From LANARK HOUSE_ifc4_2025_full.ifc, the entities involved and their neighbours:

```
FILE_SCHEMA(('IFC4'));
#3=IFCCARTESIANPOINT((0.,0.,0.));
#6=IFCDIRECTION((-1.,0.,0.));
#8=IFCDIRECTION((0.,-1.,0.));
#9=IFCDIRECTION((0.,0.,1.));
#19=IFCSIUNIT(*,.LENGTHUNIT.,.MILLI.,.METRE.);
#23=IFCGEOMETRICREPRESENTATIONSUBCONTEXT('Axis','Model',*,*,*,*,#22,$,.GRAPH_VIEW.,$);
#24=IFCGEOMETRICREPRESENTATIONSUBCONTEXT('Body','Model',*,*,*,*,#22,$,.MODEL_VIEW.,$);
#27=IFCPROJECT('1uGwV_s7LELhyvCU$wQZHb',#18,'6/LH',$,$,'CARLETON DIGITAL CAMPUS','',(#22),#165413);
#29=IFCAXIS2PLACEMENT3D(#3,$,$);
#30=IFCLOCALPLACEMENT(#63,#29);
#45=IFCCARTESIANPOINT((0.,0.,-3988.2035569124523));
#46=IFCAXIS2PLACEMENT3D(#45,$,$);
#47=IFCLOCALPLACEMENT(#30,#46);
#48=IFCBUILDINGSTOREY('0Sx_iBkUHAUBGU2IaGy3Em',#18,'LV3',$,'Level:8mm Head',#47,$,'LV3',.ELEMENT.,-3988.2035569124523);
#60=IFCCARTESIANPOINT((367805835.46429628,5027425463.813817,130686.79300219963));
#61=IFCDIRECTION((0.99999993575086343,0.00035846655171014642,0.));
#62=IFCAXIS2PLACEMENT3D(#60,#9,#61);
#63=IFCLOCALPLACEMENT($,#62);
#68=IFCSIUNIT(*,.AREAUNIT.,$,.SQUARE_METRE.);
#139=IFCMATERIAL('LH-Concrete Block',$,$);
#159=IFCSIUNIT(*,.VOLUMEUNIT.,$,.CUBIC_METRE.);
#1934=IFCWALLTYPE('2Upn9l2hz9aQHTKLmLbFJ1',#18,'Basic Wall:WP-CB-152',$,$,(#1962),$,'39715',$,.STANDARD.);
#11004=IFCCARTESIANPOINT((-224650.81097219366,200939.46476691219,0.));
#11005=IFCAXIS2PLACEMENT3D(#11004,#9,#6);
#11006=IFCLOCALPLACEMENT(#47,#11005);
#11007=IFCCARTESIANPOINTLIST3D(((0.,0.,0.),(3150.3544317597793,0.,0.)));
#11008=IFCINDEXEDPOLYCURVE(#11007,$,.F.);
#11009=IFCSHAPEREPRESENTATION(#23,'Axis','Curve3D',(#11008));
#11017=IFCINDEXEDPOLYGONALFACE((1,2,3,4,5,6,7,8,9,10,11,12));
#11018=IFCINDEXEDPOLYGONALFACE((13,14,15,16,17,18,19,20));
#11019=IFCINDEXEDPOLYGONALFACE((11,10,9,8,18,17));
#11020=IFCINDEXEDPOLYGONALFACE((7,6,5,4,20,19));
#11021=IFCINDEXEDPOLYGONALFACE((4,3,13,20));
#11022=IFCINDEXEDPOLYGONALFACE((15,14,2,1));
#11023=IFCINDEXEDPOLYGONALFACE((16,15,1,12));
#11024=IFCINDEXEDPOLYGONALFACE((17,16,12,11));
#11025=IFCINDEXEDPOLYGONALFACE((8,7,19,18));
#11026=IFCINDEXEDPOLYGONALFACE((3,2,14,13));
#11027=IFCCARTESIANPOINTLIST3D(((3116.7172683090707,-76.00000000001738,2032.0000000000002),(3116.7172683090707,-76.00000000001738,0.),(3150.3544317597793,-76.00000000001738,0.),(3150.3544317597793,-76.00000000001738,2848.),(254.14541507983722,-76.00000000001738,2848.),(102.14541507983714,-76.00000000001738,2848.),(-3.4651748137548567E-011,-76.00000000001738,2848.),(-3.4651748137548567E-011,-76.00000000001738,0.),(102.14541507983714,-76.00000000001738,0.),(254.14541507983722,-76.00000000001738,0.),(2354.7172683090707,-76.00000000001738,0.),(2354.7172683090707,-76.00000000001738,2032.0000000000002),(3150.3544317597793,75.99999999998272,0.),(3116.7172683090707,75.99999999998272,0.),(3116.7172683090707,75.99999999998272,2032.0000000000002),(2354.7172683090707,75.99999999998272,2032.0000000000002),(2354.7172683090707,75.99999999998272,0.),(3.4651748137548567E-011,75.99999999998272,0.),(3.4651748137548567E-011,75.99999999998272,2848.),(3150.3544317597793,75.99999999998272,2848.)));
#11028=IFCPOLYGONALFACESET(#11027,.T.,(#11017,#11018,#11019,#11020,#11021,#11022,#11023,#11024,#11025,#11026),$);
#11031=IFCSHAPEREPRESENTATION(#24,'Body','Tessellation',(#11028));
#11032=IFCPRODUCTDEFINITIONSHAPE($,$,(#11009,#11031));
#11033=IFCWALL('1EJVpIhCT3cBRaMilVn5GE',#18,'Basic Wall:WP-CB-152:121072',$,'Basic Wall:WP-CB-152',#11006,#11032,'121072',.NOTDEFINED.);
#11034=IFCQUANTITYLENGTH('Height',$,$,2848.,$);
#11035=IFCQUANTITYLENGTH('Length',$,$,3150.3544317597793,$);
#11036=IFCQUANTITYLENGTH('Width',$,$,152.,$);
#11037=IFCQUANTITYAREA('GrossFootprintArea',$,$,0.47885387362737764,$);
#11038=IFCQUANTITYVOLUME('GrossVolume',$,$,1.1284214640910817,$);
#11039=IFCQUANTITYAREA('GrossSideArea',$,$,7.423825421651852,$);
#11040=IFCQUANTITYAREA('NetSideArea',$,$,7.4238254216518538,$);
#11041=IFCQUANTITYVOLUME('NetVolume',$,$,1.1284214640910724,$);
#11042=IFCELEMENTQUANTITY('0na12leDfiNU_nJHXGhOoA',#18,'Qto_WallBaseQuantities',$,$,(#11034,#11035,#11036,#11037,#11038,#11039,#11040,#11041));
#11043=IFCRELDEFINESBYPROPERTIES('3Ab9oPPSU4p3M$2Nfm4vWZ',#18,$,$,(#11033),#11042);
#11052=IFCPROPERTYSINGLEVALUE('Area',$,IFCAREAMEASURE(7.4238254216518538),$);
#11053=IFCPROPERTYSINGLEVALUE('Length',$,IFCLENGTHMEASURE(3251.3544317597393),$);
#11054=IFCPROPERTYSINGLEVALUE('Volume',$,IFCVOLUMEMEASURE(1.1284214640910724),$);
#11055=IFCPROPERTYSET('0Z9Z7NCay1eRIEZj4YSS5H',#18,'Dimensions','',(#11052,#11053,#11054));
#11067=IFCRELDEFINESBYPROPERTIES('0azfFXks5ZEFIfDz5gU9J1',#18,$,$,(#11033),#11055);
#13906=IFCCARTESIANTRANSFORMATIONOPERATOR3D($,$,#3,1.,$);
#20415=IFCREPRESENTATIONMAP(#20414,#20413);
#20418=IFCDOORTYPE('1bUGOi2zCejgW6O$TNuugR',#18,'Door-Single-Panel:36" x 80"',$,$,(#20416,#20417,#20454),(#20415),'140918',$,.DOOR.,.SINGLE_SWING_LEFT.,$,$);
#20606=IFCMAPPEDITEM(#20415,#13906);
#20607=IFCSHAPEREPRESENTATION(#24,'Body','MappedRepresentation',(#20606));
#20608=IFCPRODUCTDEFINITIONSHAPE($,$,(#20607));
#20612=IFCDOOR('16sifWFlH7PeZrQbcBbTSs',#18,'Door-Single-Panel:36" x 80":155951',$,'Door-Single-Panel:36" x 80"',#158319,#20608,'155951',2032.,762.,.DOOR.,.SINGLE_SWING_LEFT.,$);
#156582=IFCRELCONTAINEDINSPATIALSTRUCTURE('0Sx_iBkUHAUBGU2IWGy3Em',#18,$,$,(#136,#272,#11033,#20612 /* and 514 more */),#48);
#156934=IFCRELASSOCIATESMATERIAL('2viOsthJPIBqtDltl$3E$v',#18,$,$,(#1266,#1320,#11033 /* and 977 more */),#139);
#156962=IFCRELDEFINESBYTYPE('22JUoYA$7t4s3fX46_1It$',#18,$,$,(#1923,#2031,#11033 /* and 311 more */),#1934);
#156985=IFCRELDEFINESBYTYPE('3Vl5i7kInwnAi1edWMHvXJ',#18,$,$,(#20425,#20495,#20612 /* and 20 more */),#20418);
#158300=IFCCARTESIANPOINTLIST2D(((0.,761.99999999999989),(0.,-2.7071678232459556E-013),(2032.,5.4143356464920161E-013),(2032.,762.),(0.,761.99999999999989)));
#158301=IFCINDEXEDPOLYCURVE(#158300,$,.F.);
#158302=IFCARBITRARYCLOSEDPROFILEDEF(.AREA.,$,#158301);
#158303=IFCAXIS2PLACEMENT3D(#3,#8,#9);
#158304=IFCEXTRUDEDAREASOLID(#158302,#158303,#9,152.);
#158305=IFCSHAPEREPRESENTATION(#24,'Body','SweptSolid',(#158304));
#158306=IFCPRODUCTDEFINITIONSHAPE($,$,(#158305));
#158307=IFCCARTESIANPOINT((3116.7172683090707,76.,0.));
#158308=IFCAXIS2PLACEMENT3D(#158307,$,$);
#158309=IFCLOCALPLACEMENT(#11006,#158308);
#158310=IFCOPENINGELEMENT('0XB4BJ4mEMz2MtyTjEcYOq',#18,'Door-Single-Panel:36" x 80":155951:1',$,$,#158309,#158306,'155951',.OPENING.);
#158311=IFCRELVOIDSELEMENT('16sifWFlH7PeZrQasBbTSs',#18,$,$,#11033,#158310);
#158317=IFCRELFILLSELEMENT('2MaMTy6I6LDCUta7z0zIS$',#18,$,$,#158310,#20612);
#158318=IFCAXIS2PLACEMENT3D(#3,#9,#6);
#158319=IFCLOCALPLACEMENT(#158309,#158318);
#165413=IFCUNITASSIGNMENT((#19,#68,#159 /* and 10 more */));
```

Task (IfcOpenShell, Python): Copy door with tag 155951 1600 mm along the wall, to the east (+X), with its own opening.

```python
import ifcopenshell
import ifcopenshell.api.feature
import ifcopenshell.api.geometry
import ifcopenshell.api.pset
import ifcopenshell.api.root
import ifcopenshell.geom
import ifcopenshell.util.element
import ifcopenshell.util.placement
import ifcopenshell.util.shape
import ifcopenshell.util.unit

model = ifcopenshell.open("LANARK HOUSE_ifc4_2025_full.ifc")
unit_scale = ifcopenshell.util.unit.calculate_unit_scale(model)
area_scale = ifcopenshell.util.unit.calculate_unit_scale(model, "AREAUNIT")
volume_scale = ifcopenshell.util.unit.calculate_unit_scale(model, "VOLUMEUNIT")
settings = ifcopenshell.geom.settings()


def volume(element):
    """Net volume in cubic metres, openings subtracted."""
    shape = ifcopenshell.geom.create_shape(settings, element)
    return ifcopenshell.util.shape.get_volume(shape.geometry)


def reuse_history(source, copy):
    """copy_class also copies each property set's owner history, people and application; keep the originals."""
    for rel in copy.IsDefinedBy:
        if rel.is_a("IfcRelDefinesByProperties") and (history := rel.RelatingPropertyDefinition.OwnerHistory):
            rel.RelatingPropertyDefinition.OwnerHistory = source.OwnerHistory
            ifcopenshell.util.element.remove_deep2(model, history)


door = model.by_guid("16sifWFlH7PeZrQbcBbTSs")
opening = door.FillsVoids[0].RelatingOpeningElement
wall = opening.VoidsElements[0].RelatingBuildingElement
before = volume(wall)
shift = ifcopenshell.util.placement.get_local_placement(wall.ObjectPlacement)[:3, 0] * -1.6 / unit_scale

# copy_class copies the void relationship, type, container and properties, but no geometry.
new_opening = ifcopenshell.api.root.copy_class(model, product=opening)
new_opening.Representation = ifcopenshell.util.element.copy_deep(
    model, opening.Representation, exclude=["IfcGeometricRepresentationContext", "IfcRepresentationMap"]
)
new_opening.Name = 'Door-Single-Panel:36" x 80"'
new_opening.Tag = None
reuse_history(opening, new_opening)
new_door = ifcopenshell.api.root.copy_class(model, product=door)
new_door.Representation = ifcopenshell.util.element.copy_deep(
    model, door.Representation, exclude=["IfcGeometricRepresentationContext", "IfcRepresentationMap"]
)
new_door.Name = 'Door-Single-Panel:36" x 80"'
new_door.Tag = None
reuse_history(door, new_door)
ifcopenshell.api.feature.add_filling(model, opening=new_opening, element=new_door)

for old, new in ((opening, new_opening), (door, new_door)):
    matrix = ifcopenshell.util.placement.get_local_placement(old.ObjectPlacement)
    matrix[:3, 3] += shift
    ifcopenshell.api.geometry.edit_object_placement(model, product=new, matrix=matrix, is_si=False)

after = volume(wall)
thickness = 0.152  # wall thickness in metres

# Update the wall's stored quantities.
qto = model.by_id(ifcopenshell.util.element.get_pset(wall, "Qto_WallBaseQuantities", should_inherit=False)["id"])
ifcopenshell.api.pset.edit_qto(model, qto=qto, properties={
    "NetSideArea": after / thickness / area_scale,
    "NetVolume": after / volume_scale,
})
pset = model.by_id(ifcopenshell.util.element.get_pset(wall, "Dimensions", should_inherit=False)["id"])
ifcopenshell.api.pset.edit_pset(model, pset=pset, properties={
    "Area": model.create_entity("IfcAreaMeasure", after / thickness / area_scale),
    "Volume": model.create_entity("IfcVolumeMeasure", after / volume_scale),
})

print(f"wall volume {before:.3f} -> {after:.3f} m3")

model.write("LANARK HOUSE_ifc4_2025_full_v2.ifc")
```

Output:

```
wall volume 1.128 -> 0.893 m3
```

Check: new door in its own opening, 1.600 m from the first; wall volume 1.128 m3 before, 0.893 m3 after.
